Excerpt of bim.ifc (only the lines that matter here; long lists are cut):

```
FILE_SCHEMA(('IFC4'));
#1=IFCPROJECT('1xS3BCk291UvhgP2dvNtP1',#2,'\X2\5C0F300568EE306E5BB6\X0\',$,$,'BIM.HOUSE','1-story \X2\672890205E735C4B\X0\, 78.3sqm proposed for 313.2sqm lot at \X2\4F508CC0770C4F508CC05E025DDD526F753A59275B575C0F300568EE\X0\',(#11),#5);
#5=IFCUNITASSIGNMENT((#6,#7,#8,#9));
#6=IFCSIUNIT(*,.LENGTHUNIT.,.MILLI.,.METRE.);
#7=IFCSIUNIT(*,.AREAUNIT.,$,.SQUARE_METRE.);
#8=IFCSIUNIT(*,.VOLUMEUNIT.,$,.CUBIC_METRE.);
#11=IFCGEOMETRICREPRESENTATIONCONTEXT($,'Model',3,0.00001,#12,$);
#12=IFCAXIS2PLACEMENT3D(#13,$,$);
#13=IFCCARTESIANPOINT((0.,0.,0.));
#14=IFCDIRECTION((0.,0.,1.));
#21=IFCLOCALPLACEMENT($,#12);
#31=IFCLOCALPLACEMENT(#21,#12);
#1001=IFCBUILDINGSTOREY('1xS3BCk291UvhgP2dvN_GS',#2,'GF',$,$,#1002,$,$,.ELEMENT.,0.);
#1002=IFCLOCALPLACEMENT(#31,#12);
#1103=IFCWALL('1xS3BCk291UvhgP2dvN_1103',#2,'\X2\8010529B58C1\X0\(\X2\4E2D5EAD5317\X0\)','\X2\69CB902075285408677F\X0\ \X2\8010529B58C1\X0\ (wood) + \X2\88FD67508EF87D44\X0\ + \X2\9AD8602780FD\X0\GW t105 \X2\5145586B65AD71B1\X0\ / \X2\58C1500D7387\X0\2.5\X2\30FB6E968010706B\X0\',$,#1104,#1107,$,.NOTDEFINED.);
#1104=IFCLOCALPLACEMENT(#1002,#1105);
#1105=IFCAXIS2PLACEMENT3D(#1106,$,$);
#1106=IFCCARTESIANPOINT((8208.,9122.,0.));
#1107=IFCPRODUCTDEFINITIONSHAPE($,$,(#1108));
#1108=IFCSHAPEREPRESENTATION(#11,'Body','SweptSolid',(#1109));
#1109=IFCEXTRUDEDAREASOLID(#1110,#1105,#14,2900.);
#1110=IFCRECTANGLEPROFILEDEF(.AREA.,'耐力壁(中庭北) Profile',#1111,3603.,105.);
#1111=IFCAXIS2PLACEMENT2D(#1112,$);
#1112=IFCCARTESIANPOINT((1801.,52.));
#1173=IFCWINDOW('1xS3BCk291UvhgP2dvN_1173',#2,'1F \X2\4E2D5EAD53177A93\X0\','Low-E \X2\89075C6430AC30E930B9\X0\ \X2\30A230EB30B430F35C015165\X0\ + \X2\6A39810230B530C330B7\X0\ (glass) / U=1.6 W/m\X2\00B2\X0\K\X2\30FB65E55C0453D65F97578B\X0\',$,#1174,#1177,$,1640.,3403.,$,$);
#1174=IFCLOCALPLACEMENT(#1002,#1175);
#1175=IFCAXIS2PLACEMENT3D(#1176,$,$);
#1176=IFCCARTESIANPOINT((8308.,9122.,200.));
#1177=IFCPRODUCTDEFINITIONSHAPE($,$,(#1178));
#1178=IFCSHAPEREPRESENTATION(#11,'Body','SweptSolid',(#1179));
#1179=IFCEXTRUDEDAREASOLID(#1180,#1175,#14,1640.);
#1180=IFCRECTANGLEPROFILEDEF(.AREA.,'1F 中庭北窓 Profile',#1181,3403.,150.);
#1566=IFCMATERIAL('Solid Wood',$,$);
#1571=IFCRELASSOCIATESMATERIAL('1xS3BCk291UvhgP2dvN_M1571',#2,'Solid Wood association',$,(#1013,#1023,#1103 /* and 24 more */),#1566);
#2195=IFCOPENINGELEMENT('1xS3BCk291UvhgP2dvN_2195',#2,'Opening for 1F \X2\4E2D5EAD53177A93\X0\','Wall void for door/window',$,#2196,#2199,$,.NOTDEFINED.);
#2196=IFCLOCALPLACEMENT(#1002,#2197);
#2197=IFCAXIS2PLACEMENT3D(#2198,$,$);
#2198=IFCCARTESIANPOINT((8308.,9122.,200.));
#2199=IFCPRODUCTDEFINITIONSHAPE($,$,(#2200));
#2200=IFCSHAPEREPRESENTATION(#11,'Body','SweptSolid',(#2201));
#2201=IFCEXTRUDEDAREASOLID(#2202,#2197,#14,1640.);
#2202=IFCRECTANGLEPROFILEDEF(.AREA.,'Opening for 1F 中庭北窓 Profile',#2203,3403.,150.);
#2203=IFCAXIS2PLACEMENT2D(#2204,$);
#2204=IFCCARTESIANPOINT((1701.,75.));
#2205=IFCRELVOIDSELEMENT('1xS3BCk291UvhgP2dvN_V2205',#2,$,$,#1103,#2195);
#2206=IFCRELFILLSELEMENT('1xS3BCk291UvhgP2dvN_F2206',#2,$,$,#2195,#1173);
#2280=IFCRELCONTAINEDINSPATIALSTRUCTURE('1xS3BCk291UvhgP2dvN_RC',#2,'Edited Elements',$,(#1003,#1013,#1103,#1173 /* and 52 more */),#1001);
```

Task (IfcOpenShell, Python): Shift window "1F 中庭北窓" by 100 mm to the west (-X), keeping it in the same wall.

```python
import ifcopenshell
import ifcopenshell.api.geometry
import ifcopenshell.util.placement
import ifcopenshell.util.unit

model = ifcopenshell.open("bim.ifc")
unit_scale = ifcopenshell.util.unit.calculate_unit_scale(model)

window = model.by_guid("1xS3BCk291UvhgP2dvN_1173")
opening = window.FillsVoids[0].RelatingOpeningElement
wall = opening.VoidsElements[0].RelatingBuildingElement

wall_matrix = ifcopenshell.util.placement.get_local_placement(wall.ObjectPlacement)
shift = wall_matrix[:3, 0] * -0.1 / unit_scale
before = ifcopenshell.util.placement.get_local_placement(window.ObjectPlacement)[:3, 3].copy()

# The window is not placed relative to its opening, so move both.
for product in (opening, window):
    matrix = ifcopenshell.util.placement.get_local_placement(product.ObjectPlacement)
    matrix[:3, 3] += shift
    ifcopenshell.api.geometry.edit_object_placement(model, product=product, matrix=matrix, is_si=False)

after = ifcopenshell.util.placement.get_local_placement(window.ObjectPlacement)[:3, 3]
print("window moved by", (after - before).round(3) + 0.0)

model.write("bim_updated.ifc")
```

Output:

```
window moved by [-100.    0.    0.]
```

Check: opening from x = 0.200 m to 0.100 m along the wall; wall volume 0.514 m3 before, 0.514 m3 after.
